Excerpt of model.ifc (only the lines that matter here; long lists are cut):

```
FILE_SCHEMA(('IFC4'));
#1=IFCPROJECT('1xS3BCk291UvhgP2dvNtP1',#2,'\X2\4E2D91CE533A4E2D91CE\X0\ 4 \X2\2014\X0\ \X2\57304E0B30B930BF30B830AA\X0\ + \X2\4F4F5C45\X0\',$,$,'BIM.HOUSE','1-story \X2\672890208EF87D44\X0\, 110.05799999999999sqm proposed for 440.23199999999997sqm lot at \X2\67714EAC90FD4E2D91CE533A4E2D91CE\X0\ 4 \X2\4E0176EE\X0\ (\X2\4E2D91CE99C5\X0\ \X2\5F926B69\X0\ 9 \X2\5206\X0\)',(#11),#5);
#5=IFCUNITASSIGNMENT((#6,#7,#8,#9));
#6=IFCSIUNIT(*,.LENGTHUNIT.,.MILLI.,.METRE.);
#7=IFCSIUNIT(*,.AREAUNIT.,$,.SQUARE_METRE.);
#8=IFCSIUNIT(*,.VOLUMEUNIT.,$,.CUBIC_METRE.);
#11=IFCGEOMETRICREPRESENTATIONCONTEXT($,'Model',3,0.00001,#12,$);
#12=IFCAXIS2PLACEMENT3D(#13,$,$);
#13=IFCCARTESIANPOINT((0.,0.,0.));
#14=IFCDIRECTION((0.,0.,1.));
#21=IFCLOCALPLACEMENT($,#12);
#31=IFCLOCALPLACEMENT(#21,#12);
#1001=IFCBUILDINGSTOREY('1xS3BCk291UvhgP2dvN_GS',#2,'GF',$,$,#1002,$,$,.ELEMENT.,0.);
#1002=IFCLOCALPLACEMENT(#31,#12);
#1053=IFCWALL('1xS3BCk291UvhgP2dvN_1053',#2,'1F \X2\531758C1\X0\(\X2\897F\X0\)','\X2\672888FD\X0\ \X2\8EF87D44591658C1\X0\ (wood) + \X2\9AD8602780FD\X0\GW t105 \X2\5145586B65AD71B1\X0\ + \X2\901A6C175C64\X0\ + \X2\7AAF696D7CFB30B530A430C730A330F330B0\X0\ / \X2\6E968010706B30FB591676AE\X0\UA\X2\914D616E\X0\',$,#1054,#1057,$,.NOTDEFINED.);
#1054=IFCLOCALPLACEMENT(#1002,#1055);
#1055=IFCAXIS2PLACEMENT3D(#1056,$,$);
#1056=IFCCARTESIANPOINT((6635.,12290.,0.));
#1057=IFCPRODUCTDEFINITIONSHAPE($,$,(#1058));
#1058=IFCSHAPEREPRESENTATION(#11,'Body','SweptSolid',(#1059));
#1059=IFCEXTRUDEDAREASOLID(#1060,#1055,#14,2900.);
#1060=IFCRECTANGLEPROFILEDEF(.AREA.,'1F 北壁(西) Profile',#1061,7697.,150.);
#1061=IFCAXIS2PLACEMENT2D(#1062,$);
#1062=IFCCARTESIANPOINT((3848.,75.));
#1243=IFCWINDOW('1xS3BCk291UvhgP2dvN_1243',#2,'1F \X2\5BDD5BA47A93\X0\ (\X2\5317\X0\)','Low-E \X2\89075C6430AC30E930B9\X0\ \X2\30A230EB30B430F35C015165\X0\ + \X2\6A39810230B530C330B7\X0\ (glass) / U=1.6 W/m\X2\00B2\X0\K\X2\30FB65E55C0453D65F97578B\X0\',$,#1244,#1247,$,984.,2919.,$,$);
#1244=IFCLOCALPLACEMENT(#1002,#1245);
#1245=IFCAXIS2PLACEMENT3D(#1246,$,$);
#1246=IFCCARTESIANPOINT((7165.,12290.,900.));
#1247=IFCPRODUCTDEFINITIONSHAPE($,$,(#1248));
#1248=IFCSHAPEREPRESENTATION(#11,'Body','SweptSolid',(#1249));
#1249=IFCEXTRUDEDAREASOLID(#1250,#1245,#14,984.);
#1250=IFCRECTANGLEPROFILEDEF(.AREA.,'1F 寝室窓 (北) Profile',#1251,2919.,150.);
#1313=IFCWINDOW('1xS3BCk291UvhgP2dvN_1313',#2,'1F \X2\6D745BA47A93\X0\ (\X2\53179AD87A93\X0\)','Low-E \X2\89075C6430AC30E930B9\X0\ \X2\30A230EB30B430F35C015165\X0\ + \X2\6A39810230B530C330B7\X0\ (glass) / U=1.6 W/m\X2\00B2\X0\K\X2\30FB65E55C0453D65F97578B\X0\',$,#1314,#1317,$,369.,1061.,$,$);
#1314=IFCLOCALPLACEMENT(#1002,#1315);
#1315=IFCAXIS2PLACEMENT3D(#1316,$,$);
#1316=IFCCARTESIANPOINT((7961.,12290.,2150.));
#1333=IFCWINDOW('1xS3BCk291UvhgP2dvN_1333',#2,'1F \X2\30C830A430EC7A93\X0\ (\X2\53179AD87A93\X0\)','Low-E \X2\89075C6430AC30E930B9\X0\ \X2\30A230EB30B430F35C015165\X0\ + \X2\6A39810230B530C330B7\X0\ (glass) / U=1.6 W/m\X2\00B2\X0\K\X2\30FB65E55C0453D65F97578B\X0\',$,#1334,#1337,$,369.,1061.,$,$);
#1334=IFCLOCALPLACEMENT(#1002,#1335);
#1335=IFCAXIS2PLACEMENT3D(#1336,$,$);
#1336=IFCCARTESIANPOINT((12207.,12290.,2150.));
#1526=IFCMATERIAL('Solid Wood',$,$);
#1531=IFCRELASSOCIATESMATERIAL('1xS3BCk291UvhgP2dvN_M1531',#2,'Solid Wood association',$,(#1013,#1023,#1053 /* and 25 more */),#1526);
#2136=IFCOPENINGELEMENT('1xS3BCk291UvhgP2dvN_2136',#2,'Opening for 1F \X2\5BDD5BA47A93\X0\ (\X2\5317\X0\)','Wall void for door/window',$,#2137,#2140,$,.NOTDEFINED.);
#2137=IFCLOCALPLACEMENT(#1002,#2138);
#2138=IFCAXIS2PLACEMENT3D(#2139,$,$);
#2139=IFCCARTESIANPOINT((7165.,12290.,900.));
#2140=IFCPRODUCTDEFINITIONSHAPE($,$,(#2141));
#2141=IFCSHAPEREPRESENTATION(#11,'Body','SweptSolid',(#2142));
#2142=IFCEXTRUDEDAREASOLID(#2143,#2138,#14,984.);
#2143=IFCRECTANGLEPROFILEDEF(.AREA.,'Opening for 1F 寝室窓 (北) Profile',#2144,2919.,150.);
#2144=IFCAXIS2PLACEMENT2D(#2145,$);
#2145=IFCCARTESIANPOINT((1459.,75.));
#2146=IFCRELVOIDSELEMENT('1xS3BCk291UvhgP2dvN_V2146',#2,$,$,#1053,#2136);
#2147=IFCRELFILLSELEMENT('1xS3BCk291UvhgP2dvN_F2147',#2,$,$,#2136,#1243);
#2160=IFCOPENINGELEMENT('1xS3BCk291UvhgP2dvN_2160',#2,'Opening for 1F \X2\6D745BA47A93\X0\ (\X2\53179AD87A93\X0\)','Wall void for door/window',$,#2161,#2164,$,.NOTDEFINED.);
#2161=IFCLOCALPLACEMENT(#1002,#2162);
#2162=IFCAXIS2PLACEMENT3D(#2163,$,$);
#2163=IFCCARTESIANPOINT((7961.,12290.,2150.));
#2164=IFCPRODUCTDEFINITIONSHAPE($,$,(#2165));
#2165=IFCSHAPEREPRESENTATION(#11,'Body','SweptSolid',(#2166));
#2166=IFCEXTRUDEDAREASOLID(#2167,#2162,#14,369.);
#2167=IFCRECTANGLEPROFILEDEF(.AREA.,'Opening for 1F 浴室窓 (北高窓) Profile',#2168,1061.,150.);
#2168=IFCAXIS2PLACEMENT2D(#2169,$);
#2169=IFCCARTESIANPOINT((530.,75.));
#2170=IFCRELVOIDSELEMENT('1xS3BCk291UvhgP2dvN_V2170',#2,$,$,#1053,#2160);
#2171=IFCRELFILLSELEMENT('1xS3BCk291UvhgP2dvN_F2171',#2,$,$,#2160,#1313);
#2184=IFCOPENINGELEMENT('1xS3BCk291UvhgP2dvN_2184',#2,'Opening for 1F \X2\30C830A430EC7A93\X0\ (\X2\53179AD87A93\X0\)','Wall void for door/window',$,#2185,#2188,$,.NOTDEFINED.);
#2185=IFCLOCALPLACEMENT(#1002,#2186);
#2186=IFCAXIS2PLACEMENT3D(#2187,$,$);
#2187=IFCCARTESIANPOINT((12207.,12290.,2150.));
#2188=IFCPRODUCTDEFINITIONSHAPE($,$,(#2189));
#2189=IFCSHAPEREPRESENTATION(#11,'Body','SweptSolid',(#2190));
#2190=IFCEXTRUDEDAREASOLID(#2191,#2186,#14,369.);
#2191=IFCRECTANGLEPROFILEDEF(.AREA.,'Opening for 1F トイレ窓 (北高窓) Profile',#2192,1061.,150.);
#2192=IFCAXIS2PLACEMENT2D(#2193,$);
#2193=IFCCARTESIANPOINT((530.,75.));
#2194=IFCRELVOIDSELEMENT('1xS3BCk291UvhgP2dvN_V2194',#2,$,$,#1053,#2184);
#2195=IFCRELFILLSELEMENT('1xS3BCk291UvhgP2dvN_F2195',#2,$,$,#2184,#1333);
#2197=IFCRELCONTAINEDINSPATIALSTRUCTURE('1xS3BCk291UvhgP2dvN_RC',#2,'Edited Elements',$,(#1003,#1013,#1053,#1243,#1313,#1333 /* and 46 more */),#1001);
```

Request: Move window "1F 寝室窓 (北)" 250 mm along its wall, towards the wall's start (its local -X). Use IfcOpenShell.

```python
import ifcopenshell
import ifcopenshell.api.geometry
import ifcopenshell.util.placement

model = ifcopenshell.open("model.ifc")

window = model.by_guid("1xS3BCk291UvhgP2dvN_1243")
opening = window.FillsVoids[0].RelatingOpeningElement
wall = opening.VoidsElements[0].RelatingBuildingElement

wall_matrix = ifcopenshell.util.placement.get_local_placement(wall.ObjectPlacement)
shift = wall_matrix[:3, 0] * -250.0
before = ifcopenshell.util.placement.get_local_placement(window.ObjectPlacement)[:3, 3].copy()

# The window is not placed relative to its opening, so move both.
for product in (opening, window):
    matrix = ifcopenshell.util.placement.get_local_placement(product.ObjectPlacement)
    matrix[:3, 3] += shift
    ifcopenshell.api.geometry.edit_object_placement(model, product=product, matrix=matrix, is_si=False)

after = ifcopenshell.util.placement.get_local_placement(window.ObjectPlacement)[:3, 3]
print("window moved by", (after - before).round(3) + 0.0)

model.write("model_updated.ifc")
```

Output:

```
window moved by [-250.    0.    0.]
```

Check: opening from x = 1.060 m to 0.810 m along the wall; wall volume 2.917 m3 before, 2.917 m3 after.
